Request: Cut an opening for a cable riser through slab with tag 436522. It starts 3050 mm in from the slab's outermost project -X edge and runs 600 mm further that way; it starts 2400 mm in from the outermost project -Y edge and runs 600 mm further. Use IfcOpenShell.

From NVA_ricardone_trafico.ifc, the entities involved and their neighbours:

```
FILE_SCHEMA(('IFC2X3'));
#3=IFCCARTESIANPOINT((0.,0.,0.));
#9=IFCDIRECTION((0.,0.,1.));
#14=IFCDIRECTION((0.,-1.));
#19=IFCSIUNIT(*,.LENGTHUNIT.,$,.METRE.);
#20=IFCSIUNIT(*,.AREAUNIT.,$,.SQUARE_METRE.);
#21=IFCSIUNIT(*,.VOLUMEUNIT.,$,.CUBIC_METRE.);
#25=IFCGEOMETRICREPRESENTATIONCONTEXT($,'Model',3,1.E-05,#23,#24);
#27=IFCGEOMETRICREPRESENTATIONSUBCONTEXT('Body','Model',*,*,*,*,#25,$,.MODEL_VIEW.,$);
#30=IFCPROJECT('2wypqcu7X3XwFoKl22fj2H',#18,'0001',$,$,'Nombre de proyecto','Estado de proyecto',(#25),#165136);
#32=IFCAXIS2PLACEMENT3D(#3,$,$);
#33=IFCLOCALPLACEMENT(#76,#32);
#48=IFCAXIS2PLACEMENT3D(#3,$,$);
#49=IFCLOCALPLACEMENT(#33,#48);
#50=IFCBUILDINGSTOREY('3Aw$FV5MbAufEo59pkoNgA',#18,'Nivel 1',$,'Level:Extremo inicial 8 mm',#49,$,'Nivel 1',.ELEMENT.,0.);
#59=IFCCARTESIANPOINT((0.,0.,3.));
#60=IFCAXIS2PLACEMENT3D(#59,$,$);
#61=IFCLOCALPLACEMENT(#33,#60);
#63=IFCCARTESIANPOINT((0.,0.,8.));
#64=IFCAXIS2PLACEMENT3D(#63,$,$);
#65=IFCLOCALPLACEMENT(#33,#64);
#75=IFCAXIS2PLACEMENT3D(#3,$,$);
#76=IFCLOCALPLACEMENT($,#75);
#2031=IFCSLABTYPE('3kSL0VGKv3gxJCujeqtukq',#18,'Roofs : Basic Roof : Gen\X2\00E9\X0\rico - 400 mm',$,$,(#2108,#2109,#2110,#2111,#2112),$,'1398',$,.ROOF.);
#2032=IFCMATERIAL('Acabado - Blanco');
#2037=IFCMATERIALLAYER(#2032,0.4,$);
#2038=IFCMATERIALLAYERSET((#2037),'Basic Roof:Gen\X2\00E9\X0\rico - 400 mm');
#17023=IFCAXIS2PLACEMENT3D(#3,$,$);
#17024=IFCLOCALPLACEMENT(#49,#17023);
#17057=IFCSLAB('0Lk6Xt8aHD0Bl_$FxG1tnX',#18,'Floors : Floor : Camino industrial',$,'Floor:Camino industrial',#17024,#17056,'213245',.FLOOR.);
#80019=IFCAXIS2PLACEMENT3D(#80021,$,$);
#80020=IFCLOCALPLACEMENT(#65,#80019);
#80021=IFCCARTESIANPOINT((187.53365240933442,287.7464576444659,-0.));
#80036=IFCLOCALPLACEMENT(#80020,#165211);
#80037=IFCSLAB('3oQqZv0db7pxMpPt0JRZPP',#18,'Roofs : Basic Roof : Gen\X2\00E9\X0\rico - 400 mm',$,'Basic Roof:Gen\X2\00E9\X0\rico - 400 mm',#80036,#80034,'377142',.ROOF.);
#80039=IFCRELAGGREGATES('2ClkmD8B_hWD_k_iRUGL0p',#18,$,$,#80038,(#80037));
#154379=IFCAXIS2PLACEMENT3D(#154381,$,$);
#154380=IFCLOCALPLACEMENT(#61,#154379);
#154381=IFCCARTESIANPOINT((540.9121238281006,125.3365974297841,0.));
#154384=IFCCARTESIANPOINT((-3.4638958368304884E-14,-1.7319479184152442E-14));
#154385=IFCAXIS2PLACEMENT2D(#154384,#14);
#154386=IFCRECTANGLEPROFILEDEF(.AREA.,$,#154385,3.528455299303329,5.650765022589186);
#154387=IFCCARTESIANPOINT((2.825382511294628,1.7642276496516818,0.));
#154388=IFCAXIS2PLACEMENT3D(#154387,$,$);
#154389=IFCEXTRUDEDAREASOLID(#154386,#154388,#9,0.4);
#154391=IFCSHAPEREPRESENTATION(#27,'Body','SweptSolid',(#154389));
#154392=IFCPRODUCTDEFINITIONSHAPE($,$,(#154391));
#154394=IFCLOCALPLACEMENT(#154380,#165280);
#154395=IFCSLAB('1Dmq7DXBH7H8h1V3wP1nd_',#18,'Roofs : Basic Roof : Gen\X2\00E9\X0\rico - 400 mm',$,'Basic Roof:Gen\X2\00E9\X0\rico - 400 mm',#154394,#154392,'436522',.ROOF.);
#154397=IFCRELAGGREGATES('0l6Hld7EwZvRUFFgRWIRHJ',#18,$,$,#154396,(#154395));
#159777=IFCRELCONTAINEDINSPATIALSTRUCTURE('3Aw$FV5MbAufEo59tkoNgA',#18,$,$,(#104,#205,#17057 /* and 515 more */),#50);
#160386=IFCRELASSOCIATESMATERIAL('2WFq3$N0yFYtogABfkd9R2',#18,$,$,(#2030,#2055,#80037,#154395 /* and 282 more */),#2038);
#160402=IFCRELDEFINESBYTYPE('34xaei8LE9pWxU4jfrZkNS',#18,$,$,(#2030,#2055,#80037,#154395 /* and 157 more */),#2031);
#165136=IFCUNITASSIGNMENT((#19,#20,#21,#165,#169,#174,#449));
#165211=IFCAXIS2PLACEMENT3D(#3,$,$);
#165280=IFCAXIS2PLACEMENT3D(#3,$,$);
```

```python
import numpy as np
import ifcopenshell
import ifcopenshell.api.feature
import ifcopenshell.api.geometry
import ifcopenshell.api.root
import ifcopenshell.geom
import ifcopenshell.util.placement
import ifcopenshell.util.representation
import ifcopenshell.util.shape
import ifcopenshell.util.unit

model = ifcopenshell.open("NVA_ricardone_trafico.ifc")
unit_scale = ifcopenshell.util.unit.calculate_unit_scale(model)
settings = ifcopenshell.geom.settings()


def volume(element):
    """Net volume in cubic metres, openings subtracted."""
    shape = ifcopenshell.geom.create_shape(settings, element)
    return ifcopenshell.util.shape.get_volume(shape.geometry)


slab = model.by_guid("1Dmq7DXBH7H8h1V3wP1nd_")
before = volume(slab)

# Extent in the slab's own axes, in metres. The edges named are its -X and -Y sides.
slab_shape = ifcopenshell.geom.create_shape(settings, slab)
vertices = ifcopenshell.util.shape.get_vertices(slab_shape.geometry)
x_min, y_min, bottom = vertices.min(axis=0)
top = vertices[:, 2].max()

opening = ifcopenshell.api.root.create_entity(model, ifc_class="IfcOpeningElement", name="Cable riser opening")
context = ifcopenshell.util.representation.get_context(model, "Model", "Body", "MODEL_VIEW")
width, depth = 0.6, 0.6
outline = [(0.0, 0.0), (width, 0.0), (width, depth), (0.0, depth), (0.0, 0.0)]
# Overshoot both faces by 50 mm so the cut is clean.
shape = ifcopenshell.api.geometry.add_slab_representation(
    model, context=context, depth=top - bottom + 0.1, polyline=outline
)
ifcopenshell.api.geometry.assign_representation(model, product=opening, representation=shape)

matrix = ifcopenshell.util.placement.get_local_placement(slab.ObjectPlacement)
matrix[:, 3] = matrix @ np.append(np.array([x_min + 3.05, y_min + 2.4, bottom - 0.05]) / unit_scale, 1.0)
ifcopenshell.api.geometry.edit_object_placement(model, product=opening, matrix=matrix, is_si=False)
ifcopenshell.api.feature.add_feature(model, feature=opening, element=slab)

after = volume(slab)

print(f"slab volume {before:.3f} -> {after:.3f} m3")

model.write("NVA_ricardone_trafico_v2.ifc")
```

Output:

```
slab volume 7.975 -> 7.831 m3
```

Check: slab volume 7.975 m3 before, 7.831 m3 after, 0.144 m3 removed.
